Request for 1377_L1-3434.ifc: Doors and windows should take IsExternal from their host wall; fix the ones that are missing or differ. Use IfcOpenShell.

First a look at what the model holds.

```python
import ifcopenshell
import ifcopenshell.util.element

model = ifcopenshell.open("1377_L1-3434.ifc")
print(model.schema)
seen = {}
for e in model.by_type("IfcDoor") + model.by_type("IfcWindow"):
    if not e.FillsVoids:
        continue
    host = e.FillsVoids[0].RelatingOpeningElement.VoidsElements[0].RelatingBuildingElement
    own = ifcopenshell.util.element.get_pset(e, f"Pset_{e.is_a()[3:].removesuffix('StandardCase')}Common", "IsExternal")
    wall = ifcopenshell.util.element.get_pset(host, "Pset_WallCommon", "IsExternal")
    seen[e.is_a(), own, wall] = seen.get((e.is_a(), own, wall), 0) + 1
for (cls, own, wall), count in sorted(seen.items(), key=str):
    print(count, cls, "IsExternal:", own, "| host wall:", wall)
```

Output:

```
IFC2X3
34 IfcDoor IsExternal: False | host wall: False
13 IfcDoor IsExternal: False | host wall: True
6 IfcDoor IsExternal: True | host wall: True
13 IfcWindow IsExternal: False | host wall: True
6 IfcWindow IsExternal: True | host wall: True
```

```python
import ifcopenshell
import ifcopenshell.api.pset
import ifcopenshell.util.element

model = ifcopenshell.open("1377_L1-3434.ifc")

count = 0
for ifc_class, pset_name in (("IfcDoor", "Pset_DoorCommon"), ("IfcWindow", "Pset_WindowCommon")):
    for e in model.by_type(ifc_class):
        if not e.FillsVoids:
            continue
        host = e.FillsVoids[0].RelatingOpeningElement.VoidsElements[0].RelatingBuildingElement
        external = ifcopenshell.util.element.get_pset(host, "Pset_WallCommon", "IsExternal")
        if external is None or ifcopenshell.util.element.get_pset(e, pset_name, "IsExternal") == external:
            continue
        pset = ifcopenshell.api.pset.add_pset(model, product=e, name=pset_name)
        ifcopenshell.api.pset.edit_pset(model, pset=pset, properties={"IsExternal": external})
        count += 1

print(count, "updated")

model.write("1377_L1-3434_edited.ifc")
```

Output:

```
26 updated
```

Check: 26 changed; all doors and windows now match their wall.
